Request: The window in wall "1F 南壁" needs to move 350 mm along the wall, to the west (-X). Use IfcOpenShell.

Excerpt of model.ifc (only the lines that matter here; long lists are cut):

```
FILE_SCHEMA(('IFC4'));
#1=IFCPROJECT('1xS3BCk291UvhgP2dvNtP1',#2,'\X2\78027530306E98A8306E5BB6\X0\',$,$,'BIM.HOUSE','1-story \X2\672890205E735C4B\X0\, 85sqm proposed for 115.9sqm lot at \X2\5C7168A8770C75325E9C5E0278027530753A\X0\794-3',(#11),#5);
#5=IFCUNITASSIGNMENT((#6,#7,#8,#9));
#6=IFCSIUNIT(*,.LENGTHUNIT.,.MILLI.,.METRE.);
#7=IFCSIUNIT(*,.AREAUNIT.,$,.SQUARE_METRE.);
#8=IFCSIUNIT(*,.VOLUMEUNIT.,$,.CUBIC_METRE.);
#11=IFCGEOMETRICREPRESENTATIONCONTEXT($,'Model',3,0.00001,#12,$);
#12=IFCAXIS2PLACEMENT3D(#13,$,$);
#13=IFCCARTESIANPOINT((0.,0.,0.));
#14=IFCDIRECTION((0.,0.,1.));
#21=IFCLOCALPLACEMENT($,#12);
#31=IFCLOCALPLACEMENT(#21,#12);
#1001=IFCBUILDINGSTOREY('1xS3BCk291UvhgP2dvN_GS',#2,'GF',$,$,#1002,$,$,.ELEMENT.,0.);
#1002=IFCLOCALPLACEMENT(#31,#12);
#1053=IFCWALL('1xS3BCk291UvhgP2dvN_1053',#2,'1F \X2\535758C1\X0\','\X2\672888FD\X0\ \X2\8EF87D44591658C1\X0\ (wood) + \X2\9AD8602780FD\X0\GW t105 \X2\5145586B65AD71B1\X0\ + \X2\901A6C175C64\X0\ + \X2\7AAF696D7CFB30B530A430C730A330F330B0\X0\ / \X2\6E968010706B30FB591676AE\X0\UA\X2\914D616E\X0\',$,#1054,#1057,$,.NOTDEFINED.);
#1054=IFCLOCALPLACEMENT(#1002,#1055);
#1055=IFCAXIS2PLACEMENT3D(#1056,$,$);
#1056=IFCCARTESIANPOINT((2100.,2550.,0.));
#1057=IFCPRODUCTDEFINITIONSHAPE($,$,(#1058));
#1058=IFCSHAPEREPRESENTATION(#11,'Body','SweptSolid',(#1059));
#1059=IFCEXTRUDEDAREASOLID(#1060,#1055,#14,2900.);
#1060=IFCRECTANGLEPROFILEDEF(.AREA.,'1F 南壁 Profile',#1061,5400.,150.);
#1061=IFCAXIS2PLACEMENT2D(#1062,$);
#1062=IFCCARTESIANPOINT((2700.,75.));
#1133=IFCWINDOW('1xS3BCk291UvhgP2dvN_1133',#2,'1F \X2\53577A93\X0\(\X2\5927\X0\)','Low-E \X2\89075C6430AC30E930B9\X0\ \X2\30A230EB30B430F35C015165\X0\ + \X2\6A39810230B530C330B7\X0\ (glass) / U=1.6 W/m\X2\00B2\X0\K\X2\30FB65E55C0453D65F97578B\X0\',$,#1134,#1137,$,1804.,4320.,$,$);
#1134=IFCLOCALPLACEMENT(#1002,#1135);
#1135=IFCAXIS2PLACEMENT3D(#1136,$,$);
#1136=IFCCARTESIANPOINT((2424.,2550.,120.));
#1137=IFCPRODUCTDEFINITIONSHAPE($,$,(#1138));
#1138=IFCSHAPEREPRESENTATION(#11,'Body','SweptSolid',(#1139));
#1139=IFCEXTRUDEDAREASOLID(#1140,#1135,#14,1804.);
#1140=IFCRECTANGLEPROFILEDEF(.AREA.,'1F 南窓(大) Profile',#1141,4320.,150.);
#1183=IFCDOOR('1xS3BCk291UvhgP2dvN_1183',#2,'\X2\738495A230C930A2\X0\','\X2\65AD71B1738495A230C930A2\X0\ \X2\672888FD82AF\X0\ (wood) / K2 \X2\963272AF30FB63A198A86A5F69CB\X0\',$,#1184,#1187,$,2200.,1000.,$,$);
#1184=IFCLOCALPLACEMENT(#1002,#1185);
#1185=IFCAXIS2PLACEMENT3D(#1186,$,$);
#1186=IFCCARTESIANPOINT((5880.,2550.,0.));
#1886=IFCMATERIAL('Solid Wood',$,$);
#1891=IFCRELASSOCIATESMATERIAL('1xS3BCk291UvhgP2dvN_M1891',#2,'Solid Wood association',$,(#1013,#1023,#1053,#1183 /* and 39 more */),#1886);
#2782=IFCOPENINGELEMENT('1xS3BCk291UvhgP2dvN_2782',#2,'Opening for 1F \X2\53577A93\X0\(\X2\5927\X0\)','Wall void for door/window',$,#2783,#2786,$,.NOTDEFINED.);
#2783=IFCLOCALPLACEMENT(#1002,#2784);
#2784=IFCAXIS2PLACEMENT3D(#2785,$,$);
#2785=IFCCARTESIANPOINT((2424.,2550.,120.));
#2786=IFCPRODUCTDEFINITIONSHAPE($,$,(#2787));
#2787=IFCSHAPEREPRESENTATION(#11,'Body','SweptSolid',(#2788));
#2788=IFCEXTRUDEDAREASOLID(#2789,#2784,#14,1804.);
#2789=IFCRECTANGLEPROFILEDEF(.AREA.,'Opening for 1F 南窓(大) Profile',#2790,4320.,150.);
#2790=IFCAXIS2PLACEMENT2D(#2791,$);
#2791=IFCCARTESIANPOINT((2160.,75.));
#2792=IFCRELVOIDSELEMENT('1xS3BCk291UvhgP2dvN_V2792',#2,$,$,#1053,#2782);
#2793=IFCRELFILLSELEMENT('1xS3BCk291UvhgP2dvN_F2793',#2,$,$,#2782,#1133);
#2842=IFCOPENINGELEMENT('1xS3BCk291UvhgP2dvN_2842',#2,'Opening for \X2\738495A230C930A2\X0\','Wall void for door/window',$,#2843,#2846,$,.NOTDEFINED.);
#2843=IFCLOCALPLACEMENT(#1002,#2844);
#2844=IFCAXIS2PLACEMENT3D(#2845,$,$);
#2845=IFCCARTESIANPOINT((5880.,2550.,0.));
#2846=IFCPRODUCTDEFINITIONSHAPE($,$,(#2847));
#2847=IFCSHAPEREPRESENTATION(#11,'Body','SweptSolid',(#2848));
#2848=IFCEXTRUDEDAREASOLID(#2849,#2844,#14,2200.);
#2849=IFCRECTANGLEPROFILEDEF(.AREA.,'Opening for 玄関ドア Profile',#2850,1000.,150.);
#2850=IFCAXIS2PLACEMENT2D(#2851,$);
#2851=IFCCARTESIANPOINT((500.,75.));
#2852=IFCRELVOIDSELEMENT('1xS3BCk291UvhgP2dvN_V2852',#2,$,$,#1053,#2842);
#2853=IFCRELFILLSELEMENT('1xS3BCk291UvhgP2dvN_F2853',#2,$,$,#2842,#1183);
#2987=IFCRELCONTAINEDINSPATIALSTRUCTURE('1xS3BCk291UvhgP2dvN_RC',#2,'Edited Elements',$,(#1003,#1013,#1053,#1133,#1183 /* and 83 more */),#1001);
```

```python
import ifcopenshell
import ifcopenshell.api.geometry
import ifcopenshell.util.placement

model = ifcopenshell.open("model.ifc")

window = model.by_id(1133)
opening = window.FillsVoids[0].RelatingOpeningElement
wall = opening.VoidsElements[0].RelatingBuildingElement

wall_matrix = ifcopenshell.util.placement.get_local_placement(wall.ObjectPlacement)
shift = wall_matrix[:3, 0] * -350.0
before = ifcopenshell.util.placement.get_local_placement(window.ObjectPlacement)[:3, 3].copy()

# The window is not placed relative to its opening, so move both.
for product in (opening, window):
    matrix = ifcopenshell.util.placement.get_local_placement(product.ObjectPlacement)
    matrix[:3, 3] += shift
    ifcopenshell.api.geometry.edit_object_placement(model, product=product, matrix=matrix, is_si=False)

after = ifcopenshell.util.placement.get_local_placement(window.ObjectPlacement)[:3, 3]
print("window moved by", (after - before).round(3) + 0.0)

model.write("model_rev.ifc")
```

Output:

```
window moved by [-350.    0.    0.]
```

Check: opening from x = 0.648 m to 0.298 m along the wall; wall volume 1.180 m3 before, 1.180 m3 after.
